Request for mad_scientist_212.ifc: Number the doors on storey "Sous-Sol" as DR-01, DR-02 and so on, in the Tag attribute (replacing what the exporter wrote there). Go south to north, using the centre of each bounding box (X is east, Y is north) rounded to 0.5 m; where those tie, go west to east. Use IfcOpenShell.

First a look at what the model holds.

```python
import ifcopenshell
import ifcopenshell.util.element
import ifcopenshell.util.placement

model = ifcopenshell.open("mad_scientist_212.ifc")
print(model.schema)
storey = next(s for s in model.by_type("IfcBuildingStorey") if s.Name == "Sous-Sol")
doors = [e for e in ifcopenshell.util.element.get_decomposition(storey) if e.is_a("IfcDoor")]
for e in sorted(doors, key=lambda e: e.id()):
    origin = ifcopenshell.util.placement.get_local_placement(e.ObjectPlacement)[:3, 3]
    print(e.id(), e.Tag, e.Name, origin.round(2) + 0.0, sep=" | ")
```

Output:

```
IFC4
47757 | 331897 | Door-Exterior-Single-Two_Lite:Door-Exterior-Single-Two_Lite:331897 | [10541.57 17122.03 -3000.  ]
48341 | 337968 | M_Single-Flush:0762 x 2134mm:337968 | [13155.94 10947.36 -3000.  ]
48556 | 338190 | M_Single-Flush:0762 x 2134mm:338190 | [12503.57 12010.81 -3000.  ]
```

```python
import ifcopenshell
import ifcopenshell.geom
import ifcopenshell.util.element
import ifcopenshell.util.shape

model = ifcopenshell.open("mad_scientist_212.ifc")
settings = ifcopenshell.geom.settings()
settings.set("use-world-coords", True)


def centre(element):
    shape = ifcopenshell.geom.create_shape(settings, element)
    return ifcopenshell.util.shape.get_bbox_centroid(shape.geometry)


storey = next(s for s in model.by_type("IfcBuildingStorey") if s.Name == "Sous-Sol")
doors = [e for e in ifcopenshell.util.element.get_decomposition(storey) if e.is_a("IfcDoor")]

# Insertion points can sit at a corner or the storey origin, so sort by the geometry (in metres).
centres = {e: centre(e) for e in doors}
doors.sort(key=lambda e: (round(centres[e][1] / 0.5), centres[e][0]))

for i, e in enumerate(doors, start=1):
    number = f"DR-{i:02d}"
    e.Tag = number
    print(e.id(), number)

model.write("mad_scientist_212_rev.ifc")
```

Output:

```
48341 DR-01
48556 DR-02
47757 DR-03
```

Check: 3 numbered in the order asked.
